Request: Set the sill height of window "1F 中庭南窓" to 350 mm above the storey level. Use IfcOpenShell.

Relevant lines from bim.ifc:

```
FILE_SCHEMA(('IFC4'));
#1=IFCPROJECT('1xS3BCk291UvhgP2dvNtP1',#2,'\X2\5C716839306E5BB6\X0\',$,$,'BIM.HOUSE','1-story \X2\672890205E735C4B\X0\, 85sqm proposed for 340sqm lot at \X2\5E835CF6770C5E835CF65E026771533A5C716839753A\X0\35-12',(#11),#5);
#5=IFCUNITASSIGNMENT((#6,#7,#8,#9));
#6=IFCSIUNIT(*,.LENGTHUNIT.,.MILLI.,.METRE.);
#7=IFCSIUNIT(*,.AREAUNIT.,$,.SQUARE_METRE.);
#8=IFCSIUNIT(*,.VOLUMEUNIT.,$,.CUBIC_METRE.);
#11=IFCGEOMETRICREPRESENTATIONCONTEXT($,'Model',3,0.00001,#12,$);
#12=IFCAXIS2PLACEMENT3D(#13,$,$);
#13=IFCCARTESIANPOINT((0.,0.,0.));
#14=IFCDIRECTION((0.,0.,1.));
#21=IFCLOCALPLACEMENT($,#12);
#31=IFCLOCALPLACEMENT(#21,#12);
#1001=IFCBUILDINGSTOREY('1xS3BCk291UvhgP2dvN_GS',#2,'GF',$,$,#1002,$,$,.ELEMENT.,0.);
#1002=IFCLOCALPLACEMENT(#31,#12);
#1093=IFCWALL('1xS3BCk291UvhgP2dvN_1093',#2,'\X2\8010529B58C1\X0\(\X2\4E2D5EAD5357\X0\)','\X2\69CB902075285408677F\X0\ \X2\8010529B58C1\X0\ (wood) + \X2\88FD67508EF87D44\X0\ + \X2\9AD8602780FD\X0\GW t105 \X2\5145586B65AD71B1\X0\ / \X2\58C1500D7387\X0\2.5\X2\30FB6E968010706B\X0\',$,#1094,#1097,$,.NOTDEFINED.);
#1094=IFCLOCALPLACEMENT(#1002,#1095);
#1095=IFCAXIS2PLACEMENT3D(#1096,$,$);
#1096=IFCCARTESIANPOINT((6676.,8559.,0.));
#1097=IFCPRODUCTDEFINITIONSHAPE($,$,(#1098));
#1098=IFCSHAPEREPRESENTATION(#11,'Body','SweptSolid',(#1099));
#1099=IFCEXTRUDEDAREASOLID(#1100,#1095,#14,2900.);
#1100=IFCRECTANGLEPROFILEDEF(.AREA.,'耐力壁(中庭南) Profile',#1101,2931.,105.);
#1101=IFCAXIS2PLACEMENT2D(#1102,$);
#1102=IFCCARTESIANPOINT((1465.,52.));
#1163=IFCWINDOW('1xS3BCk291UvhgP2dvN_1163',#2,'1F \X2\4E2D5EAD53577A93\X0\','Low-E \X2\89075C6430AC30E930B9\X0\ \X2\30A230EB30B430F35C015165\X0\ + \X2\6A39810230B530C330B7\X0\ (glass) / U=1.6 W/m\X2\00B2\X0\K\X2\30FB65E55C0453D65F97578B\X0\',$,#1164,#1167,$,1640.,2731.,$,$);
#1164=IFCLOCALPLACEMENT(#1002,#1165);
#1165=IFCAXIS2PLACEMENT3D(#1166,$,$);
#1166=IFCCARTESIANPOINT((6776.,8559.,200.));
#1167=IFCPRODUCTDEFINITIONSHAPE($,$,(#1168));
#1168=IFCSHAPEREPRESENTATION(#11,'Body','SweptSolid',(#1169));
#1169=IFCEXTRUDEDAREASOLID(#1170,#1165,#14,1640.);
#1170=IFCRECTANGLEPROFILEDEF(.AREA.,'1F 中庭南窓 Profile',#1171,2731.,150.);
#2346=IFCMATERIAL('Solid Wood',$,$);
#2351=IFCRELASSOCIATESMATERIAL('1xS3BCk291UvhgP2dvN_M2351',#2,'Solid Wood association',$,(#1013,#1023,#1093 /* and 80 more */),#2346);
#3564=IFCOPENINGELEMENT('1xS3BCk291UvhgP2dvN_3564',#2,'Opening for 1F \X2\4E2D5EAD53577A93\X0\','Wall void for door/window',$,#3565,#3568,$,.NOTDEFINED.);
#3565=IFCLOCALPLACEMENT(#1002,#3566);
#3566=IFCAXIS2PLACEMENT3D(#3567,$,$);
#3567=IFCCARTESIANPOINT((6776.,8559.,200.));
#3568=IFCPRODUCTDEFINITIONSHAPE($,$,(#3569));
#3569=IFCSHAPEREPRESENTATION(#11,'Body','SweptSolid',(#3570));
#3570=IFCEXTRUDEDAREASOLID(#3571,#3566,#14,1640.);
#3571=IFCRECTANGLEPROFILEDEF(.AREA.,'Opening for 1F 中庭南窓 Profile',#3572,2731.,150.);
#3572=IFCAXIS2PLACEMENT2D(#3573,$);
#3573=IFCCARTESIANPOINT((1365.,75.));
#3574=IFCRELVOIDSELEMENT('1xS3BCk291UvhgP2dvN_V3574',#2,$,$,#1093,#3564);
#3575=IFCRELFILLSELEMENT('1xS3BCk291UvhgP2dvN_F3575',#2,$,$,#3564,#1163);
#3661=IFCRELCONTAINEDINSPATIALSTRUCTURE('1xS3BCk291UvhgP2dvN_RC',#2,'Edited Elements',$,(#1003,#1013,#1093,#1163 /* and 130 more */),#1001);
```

```python
import numpy as np
import ifcopenshell
import ifcopenshell.api.geometry
import ifcopenshell.geom
import ifcopenshell.util.element
import ifcopenshell.util.placement
import ifcopenshell.util.shape
import ifcopenshell.util.unit

model = ifcopenshell.open("bim.ifc")
unit_scale = ifcopenshell.util.unit.calculate_unit_scale(model)

window = model.by_guid("1xS3BCk291UvhgP2dvN_1163")
opening = window.FillsVoids[0].RelatingOpeningElement
storey = ifcopenshell.util.element.get_container(window, ifc_class="IfcBuildingStorey")
level = ifcopenshell.util.placement.get_local_placement(storey.ObjectPlacement)[2, 3]

# The opening's origin need not be at the sill, so measure its lowest point.
shape = ifcopenshell.geom.create_shape(ifcopenshell.geom.settings(), opening)
bottom = ifcopenshell.util.shape.get_shape_bottom_elevation(shape, shape.geometry) / unit_scale
dz = level + 0.35 / unit_scale - bottom

shift = np.array([0.0, 0.0, dz])
# The window is not placed relative to its opening, so move both.
for product in (opening, window):
    matrix = ifcopenshell.util.placement.get_local_placement(product.ObjectPlacement)
    matrix[:3, 3] += shift
    ifcopenshell.api.geometry.edit_object_placement(model, product=product, matrix=matrix, is_si=False)

print(f"moved by {dz * unit_scale:+.3f} m")

model.write("bim_v2.ifc")
```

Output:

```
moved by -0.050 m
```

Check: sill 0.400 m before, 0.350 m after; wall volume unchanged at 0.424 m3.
